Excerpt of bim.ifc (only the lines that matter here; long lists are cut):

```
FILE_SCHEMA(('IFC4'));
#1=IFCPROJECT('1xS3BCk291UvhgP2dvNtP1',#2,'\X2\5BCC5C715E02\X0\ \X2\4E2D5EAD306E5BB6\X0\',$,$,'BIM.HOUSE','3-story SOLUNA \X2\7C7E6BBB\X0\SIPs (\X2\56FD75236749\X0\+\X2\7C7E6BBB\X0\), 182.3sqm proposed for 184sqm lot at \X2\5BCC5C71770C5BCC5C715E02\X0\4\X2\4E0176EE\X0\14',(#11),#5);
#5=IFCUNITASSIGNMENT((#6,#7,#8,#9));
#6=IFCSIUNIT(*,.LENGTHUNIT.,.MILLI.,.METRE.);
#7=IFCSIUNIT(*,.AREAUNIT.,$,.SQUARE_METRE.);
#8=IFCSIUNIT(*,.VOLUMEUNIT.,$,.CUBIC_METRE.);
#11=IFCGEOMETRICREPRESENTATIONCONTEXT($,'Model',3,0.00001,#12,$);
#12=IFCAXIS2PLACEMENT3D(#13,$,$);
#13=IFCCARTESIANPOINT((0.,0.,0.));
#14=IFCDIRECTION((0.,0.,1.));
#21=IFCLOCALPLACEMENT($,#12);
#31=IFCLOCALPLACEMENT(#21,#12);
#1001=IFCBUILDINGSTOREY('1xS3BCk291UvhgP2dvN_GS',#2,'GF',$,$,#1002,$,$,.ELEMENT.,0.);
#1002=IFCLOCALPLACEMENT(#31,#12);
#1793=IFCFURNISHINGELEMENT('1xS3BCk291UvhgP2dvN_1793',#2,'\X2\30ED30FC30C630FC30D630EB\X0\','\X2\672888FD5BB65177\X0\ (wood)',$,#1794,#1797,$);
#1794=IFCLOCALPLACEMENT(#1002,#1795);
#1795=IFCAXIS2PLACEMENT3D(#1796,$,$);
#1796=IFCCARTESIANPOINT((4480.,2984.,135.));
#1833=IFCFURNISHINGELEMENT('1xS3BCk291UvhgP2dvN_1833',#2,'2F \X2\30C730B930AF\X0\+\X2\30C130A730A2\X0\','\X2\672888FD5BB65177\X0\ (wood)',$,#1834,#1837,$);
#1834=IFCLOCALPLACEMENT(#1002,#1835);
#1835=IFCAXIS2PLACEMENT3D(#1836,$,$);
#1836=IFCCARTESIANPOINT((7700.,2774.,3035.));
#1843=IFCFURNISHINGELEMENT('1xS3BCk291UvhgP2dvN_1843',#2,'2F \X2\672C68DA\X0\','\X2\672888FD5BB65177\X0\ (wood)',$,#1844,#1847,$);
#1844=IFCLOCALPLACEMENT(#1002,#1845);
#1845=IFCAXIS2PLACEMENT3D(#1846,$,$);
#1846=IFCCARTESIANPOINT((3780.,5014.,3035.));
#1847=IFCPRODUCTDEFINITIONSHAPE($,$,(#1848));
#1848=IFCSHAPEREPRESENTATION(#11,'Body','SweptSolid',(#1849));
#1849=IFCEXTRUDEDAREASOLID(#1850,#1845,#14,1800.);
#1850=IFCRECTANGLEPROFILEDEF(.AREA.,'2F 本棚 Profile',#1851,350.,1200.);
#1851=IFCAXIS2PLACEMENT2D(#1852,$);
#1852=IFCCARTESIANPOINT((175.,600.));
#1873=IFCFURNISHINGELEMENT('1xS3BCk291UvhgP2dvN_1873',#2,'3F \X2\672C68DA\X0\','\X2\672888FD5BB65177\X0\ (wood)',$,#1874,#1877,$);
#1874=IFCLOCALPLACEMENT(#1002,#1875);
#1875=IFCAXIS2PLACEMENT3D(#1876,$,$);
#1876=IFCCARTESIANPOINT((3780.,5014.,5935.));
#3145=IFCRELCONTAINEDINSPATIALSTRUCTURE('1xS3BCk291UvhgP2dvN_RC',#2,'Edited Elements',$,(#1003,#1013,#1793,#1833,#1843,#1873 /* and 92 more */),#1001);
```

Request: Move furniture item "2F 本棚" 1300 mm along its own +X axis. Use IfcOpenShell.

```python
import ifcopenshell
import ifcopenshell.api.geometry
import ifcopenshell.util.placement
import ifcopenshell.util.unit

model = ifcopenshell.open("bim.ifc")
unit_scale = ifcopenshell.util.unit.calculate_unit_scale(model)

item = model.by_id(1843)
matrix = ifcopenshell.util.placement.get_local_placement(item.ObjectPlacement)
matrix[:3, 3] += matrix[:3, 0] * 1.3 / unit_scale
ifcopenshell.api.geometry.edit_object_placement(model, product=item, matrix=matrix, is_si=False)

print(ifcopenshell.util.placement.get_local_placement(item.ObjectPlacement).round(3) + 0.0)

model.write("bim_edited.ifc")
```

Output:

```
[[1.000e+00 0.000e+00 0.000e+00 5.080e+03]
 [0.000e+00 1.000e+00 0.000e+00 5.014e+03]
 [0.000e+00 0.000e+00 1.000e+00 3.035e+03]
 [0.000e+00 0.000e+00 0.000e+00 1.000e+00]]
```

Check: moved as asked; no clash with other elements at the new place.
